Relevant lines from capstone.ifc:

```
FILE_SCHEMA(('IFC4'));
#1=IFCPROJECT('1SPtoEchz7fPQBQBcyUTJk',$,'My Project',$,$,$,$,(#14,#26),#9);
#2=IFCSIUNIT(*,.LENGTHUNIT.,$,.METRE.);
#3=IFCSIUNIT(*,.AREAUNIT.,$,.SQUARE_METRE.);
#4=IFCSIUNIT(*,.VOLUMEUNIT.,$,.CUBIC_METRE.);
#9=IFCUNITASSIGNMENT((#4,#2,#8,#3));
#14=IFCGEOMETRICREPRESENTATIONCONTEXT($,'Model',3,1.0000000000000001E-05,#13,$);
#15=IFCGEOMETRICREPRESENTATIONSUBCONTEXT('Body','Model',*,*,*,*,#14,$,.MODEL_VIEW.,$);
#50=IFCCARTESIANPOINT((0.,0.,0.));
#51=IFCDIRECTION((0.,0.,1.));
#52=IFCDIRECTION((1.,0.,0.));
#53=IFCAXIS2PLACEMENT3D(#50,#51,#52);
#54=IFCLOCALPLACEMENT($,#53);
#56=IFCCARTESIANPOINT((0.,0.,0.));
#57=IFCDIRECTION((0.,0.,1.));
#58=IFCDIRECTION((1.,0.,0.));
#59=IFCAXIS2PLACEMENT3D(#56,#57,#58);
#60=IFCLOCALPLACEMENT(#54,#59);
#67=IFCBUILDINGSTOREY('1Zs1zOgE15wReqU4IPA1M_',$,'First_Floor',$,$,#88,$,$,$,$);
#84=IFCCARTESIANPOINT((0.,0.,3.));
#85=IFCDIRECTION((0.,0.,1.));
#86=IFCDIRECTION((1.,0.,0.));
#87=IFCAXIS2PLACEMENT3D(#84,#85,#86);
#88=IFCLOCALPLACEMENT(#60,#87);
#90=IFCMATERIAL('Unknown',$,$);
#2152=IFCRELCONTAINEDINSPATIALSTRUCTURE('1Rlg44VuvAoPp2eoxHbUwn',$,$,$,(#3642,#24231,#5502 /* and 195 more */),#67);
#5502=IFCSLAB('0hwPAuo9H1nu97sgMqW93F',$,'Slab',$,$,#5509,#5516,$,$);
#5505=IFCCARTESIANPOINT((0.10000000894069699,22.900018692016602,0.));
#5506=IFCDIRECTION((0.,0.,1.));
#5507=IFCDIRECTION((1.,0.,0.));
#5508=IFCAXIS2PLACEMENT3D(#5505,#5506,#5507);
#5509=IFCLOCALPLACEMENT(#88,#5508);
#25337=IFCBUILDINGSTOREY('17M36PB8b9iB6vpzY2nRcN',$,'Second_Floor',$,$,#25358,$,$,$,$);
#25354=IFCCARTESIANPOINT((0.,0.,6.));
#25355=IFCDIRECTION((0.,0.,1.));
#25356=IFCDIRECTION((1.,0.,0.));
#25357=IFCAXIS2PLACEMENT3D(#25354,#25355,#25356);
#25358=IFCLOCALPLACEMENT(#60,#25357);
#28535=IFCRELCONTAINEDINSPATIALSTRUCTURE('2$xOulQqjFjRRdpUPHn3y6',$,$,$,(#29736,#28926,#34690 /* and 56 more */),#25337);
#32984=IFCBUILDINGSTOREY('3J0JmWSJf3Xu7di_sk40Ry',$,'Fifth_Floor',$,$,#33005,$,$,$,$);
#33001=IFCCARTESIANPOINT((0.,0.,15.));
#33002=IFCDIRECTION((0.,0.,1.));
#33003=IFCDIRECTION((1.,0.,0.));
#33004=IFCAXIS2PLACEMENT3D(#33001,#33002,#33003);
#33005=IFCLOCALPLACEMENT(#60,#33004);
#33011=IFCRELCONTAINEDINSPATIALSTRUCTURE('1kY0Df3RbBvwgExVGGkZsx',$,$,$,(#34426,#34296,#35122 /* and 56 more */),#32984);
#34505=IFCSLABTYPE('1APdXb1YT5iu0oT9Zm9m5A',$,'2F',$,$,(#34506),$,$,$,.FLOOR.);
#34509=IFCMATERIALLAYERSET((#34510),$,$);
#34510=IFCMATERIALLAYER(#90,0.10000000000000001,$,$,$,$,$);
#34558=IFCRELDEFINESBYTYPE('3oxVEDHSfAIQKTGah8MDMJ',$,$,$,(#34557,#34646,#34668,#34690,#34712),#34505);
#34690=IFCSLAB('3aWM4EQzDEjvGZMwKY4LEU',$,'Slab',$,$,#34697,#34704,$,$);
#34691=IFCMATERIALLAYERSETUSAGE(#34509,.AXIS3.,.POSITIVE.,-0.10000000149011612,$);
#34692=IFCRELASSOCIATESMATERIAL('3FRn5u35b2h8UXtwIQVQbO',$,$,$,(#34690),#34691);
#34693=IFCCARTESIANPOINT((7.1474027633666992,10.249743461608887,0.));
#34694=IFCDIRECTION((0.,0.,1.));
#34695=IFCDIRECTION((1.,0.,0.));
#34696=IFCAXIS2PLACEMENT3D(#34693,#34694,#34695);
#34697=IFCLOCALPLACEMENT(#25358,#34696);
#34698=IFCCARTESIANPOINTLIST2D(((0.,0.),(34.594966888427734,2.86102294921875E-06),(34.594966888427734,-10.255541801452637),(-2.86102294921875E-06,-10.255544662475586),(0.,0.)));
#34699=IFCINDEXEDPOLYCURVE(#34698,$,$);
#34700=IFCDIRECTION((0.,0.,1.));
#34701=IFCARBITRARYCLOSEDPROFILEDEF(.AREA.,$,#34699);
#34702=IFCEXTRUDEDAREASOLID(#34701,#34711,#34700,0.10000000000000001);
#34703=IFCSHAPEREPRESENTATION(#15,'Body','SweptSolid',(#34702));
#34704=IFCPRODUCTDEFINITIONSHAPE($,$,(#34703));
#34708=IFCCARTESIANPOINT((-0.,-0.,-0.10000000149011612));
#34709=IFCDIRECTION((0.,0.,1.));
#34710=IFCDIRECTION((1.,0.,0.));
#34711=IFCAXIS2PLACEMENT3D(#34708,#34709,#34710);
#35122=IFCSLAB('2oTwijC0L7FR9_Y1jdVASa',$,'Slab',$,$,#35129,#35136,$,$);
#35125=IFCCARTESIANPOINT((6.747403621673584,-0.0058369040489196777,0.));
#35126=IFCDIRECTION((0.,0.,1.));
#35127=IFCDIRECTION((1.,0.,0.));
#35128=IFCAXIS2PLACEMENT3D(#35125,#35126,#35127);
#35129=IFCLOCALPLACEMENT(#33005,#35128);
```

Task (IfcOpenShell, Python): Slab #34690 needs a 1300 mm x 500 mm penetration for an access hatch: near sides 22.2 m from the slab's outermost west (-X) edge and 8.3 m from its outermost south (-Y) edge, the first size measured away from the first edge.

```python
import numpy as np
import ifcopenshell
import ifcopenshell.api.feature
import ifcopenshell.api.geometry
import ifcopenshell.api.root
import ifcopenshell.geom
import ifcopenshell.util.placement
import ifcopenshell.util.representation
import ifcopenshell.util.shape
import ifcopenshell.util.unit

model = ifcopenshell.open("capstone.ifc")
unit_scale = ifcopenshell.util.unit.calculate_unit_scale(model)
settings = ifcopenshell.geom.settings()


def volume(element):
    """Net volume in cubic metres, openings subtracted."""
    shape = ifcopenshell.geom.create_shape(settings, element)
    return ifcopenshell.util.shape.get_volume(shape.geometry)


slab = model.by_id(34690)
before = volume(slab)

# Extent in the slab's own axes, in metres. The edges named are its -X and -Y sides.
slab_shape = ifcopenshell.geom.create_shape(settings, slab)
vertices = ifcopenshell.util.shape.get_vertices(slab_shape.geometry)
x_min, y_min, bottom = vertices.min(axis=0)
top = vertices[:, 2].max()

opening = ifcopenshell.api.root.create_entity(model, ifc_class="IfcOpeningElement", name="Access hatch opening", predefined_type="OPENING")
context = ifcopenshell.util.representation.get_context(model, "Model", "Body", "MODEL_VIEW")
width, depth = 1.3, 0.5
outline = [(0.0, 0.0), (width, 0.0), (width, depth), (0.0, depth), (0.0, 0.0)]
# Overshoot both faces by 50 mm so the cut is clean.
shape = ifcopenshell.api.geometry.add_slab_representation(
    model, context=context, depth=top - bottom + 0.1, polyline=outline
)
ifcopenshell.api.geometry.assign_representation(model, product=opening, representation=shape)

matrix = ifcopenshell.util.placement.get_local_placement(slab.ObjectPlacement)
matrix[:, 3] = matrix @ np.append(np.array([x_min + 22.2, y_min + 8.3, bottom - 0.05]) / unit_scale, 1.0)
ifcopenshell.api.geometry.edit_object_placement(model, product=opening, matrix=matrix, is_si=False)
ifcopenshell.api.feature.add_feature(model, feature=opening, element=slab)

after = volume(slab)

print(f"slab volume {before:.3f} -> {after:.3f} m3")

model.write("capstone_v2.ifc")
```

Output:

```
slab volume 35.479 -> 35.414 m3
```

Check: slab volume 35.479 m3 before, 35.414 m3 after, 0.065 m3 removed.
